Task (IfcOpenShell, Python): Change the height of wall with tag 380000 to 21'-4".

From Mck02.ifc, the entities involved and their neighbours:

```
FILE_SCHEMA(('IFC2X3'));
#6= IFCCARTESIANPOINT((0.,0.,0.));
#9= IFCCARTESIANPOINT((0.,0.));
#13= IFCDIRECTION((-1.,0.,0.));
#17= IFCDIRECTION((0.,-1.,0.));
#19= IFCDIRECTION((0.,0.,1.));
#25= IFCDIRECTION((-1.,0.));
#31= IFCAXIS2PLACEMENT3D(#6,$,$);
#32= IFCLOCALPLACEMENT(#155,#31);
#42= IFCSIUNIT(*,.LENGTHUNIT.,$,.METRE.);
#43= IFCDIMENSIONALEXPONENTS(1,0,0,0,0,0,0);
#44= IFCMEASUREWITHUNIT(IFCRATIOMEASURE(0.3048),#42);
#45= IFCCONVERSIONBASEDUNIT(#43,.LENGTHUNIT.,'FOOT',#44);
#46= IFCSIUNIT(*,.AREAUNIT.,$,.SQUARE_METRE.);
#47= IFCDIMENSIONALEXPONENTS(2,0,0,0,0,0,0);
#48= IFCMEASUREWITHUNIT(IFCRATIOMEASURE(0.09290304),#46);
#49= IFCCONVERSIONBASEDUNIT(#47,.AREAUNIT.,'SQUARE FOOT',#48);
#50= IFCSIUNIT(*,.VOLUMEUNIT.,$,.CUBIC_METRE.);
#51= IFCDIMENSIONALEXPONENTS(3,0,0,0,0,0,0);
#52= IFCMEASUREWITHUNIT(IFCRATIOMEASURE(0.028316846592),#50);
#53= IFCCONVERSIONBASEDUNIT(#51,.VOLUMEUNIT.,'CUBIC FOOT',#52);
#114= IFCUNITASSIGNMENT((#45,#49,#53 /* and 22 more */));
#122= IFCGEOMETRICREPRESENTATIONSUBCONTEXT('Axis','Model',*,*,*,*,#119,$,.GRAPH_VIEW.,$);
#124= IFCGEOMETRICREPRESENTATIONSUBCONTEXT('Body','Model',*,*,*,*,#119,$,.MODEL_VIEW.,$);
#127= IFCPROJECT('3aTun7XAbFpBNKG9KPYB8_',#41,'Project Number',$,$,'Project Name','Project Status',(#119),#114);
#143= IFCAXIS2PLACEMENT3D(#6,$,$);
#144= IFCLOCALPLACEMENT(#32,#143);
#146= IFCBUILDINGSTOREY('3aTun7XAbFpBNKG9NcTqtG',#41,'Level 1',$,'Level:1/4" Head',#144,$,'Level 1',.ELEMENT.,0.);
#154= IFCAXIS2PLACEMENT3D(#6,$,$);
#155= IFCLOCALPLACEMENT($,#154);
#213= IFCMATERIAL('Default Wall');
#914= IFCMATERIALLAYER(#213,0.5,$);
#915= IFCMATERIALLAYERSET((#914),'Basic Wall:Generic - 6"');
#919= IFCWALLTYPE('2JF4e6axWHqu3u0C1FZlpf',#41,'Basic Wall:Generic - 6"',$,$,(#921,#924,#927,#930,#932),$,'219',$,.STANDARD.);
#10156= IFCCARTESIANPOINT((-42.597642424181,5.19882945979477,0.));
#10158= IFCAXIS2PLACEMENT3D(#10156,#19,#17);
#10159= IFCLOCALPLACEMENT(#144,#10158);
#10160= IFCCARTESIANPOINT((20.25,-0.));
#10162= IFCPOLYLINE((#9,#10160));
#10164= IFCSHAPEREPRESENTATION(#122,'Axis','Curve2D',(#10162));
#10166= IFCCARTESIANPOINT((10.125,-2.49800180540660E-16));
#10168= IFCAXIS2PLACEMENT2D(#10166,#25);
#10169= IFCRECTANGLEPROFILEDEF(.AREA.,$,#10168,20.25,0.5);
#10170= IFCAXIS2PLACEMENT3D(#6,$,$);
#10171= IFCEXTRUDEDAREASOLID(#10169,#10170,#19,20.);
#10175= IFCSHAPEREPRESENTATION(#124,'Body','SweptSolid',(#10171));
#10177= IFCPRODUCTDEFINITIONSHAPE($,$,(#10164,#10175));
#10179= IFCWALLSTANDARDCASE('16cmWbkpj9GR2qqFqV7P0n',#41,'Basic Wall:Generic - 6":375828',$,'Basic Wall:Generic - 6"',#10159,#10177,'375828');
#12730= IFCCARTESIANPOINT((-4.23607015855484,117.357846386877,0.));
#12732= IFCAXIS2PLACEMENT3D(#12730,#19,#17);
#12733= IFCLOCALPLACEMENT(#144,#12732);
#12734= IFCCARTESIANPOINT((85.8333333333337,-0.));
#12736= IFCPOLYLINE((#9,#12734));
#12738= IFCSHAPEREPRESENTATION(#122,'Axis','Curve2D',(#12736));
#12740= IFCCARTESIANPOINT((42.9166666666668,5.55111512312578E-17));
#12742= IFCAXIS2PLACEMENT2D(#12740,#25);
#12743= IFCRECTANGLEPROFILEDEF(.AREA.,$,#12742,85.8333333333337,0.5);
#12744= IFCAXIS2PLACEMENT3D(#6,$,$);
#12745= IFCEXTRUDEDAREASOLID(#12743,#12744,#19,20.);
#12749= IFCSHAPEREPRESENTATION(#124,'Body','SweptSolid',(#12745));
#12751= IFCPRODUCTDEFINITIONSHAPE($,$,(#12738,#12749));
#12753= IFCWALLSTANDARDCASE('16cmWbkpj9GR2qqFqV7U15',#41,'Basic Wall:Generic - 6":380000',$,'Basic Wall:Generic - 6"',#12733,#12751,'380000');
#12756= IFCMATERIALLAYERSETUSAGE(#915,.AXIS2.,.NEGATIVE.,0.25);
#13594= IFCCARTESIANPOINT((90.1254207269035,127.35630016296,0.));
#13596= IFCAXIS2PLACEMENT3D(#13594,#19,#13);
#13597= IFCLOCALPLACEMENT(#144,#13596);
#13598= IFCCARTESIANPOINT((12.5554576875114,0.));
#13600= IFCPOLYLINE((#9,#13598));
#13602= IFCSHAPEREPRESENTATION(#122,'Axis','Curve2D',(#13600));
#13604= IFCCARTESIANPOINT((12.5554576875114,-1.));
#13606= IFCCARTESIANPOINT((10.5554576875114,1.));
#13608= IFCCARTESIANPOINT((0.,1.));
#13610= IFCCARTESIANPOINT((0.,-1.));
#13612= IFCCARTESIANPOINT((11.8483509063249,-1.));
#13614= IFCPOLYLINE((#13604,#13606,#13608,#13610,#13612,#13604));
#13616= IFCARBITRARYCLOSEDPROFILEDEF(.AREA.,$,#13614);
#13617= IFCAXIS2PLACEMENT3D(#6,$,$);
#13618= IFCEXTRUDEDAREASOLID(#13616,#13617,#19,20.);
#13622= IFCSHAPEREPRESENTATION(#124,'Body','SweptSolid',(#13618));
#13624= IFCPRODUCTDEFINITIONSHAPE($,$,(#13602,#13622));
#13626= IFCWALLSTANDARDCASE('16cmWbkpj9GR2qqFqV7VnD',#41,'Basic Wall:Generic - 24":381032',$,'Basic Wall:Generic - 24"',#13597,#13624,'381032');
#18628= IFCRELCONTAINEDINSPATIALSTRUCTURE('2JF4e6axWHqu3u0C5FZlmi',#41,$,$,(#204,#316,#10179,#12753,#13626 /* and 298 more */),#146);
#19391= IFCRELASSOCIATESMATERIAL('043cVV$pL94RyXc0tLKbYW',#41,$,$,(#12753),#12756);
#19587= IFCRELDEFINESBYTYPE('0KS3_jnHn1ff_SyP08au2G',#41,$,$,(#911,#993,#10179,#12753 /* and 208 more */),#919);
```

```python
import ifcopenshell
import ifcopenshell.geom
import ifcopenshell.util.representation
import ifcopenshell.util.shape
import ifcopenshell.util.unit

model = ifcopenshell.open("Mck02.ifc")
unit_scale = ifcopenshell.util.unit.calculate_unit_scale(model)
settings = ifcopenshell.geom.settings()


def volume(element):
    """Net volume in cubic metres, openings subtracted."""
    shape = ifcopenshell.geom.create_shape(settings, element)
    return ifcopenshell.util.shape.get_volume(shape.geometry)


wall = model.by_guid("16cmWbkpj9GR2qqFqV7U15")
before = volume(wall)

body = ifcopenshell.util.representation.get_representation(wall, "Model", "Body")
solid = body.Items[0]
old_height = solid.Depth
solid.Depth = 256 * 0.0254 / unit_scale
after = volume(wall)

print(f"height {old_height:g} -> {solid.Depth:g}, volume {before:.3f} -> {after:.3f} m3")

model.write("Mck02_rev.ifc")
```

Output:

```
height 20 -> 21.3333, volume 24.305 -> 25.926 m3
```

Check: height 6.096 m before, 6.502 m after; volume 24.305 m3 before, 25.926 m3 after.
